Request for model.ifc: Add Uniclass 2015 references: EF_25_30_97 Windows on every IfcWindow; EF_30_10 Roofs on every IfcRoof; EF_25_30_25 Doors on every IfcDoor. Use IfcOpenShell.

First a look at what the model holds.

```python
import ifcopenshell

model = ifcopenshell.open("model.ifc")
print(model.schema)
print("classifications:", [c.Name for c in model.by_type("IfcClassification")])
for ifc_class in ("IfcDoor", "IfcRoof", "IfcStair", "IfcWall", "IfcWindow"):
    print(ifc_class, len(model.by_type(ifc_class)))
```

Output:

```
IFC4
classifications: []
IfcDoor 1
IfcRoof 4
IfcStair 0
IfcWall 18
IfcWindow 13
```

```python
import ifcopenshell
import ifcopenshell.api.classification

model = ifcopenshell.open("model.ifc")

system = ifcopenshell.api.classification.add_classification(model, classification="Uniclass 2015")

codes = {
    "IfcWindow": ("EF_25_30_97", "Windows"),
    "IfcRoof": ("EF_30_10", "Roofs"),
    "IfcDoor": ("EF_25_30_25", "Doors"),
}
for ifc_class, (code, name) in codes.items():
    products = model.by_type(ifc_class)
    ifcopenshell.api.classification.add_reference(
        model, products=products, classification=system, identification=code, name=name
    )
    print(code, len(products))

model.write("model-out.ifc")
```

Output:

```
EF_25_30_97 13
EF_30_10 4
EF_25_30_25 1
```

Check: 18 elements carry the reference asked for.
